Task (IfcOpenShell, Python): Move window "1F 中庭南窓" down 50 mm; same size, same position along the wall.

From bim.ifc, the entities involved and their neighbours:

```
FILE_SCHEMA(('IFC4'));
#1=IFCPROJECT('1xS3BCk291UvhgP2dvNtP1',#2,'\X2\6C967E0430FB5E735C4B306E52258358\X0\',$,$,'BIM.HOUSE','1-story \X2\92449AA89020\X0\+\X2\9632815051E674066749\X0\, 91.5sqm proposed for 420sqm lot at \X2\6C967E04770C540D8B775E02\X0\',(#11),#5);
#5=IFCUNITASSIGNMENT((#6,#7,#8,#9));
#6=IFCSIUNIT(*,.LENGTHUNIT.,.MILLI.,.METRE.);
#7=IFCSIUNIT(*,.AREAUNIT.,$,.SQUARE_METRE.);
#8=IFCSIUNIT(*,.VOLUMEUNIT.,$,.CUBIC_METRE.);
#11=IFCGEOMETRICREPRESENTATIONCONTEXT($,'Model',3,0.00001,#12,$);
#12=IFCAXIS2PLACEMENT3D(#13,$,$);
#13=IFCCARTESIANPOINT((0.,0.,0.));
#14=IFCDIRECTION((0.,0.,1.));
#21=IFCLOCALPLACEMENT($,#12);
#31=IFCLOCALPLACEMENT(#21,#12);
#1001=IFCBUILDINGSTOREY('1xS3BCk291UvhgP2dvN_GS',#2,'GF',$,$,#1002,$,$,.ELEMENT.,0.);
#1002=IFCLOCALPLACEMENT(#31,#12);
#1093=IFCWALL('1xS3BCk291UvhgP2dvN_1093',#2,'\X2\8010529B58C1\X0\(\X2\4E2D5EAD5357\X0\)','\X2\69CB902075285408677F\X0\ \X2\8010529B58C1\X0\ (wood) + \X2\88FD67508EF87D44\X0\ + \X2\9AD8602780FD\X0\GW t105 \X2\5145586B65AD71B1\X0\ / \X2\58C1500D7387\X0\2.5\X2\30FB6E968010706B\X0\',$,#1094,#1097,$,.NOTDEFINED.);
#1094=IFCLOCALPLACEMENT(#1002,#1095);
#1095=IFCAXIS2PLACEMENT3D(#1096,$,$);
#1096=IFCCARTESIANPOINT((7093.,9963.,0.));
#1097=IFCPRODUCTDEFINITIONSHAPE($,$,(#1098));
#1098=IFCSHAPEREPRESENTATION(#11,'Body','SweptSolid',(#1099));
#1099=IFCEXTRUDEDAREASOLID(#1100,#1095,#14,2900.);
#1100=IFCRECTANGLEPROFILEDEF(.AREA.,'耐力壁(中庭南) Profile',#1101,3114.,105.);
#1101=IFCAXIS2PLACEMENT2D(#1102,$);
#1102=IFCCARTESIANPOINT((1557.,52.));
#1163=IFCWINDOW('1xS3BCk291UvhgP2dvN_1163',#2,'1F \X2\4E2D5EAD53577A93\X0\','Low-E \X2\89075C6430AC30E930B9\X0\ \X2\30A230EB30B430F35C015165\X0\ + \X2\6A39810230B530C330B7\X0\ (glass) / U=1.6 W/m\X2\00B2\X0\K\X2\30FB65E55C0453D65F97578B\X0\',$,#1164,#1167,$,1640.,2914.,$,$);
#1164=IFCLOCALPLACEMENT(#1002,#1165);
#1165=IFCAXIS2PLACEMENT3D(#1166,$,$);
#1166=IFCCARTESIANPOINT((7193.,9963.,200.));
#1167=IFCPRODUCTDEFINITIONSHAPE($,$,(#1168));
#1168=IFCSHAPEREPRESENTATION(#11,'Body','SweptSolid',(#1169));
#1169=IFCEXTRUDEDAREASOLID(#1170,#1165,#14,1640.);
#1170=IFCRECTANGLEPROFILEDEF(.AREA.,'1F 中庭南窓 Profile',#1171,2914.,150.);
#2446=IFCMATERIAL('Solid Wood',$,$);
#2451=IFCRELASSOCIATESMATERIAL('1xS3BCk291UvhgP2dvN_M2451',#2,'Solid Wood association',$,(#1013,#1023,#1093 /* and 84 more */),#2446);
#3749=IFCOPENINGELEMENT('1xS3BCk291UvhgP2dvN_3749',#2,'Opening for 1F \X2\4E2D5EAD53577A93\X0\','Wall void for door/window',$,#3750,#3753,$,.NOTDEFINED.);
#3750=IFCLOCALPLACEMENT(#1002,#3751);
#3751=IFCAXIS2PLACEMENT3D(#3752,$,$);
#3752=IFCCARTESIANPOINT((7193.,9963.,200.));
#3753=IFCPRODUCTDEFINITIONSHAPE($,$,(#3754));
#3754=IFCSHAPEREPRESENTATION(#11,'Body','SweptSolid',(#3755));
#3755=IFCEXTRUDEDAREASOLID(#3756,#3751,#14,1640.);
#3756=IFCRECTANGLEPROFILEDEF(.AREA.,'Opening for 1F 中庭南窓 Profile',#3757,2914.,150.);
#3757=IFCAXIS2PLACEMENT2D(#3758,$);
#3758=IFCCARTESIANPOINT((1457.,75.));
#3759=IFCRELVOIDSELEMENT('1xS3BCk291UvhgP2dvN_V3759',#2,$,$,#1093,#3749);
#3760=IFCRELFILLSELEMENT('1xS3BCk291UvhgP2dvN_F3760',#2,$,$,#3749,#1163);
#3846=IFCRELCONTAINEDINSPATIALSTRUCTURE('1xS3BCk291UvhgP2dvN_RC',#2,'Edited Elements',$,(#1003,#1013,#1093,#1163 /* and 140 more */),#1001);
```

```python
import numpy as np
import ifcopenshell
import ifcopenshell.api.geometry
import ifcopenshell.util.placement
import ifcopenshell.util.unit

model = ifcopenshell.open("bim.ifc")
unit_scale = ifcopenshell.util.unit.calculate_unit_scale(model)

window = model.by_guid("1xS3BCk291UvhgP2dvN_1163")
opening = window.FillsVoids[0].RelatingOpeningElement
dz = -0.05 / unit_scale

shift = np.array([0.0, 0.0, dz])
# The window is not placed relative to its opening, so move both.
for product in (opening, window):
    matrix = ifcopenshell.util.placement.get_local_placement(product.ObjectPlacement)
    matrix[:3, 3] += shift
    ifcopenshell.api.geometry.edit_object_placement(model, product=product, matrix=matrix, is_si=False)

print(f"moved by {dz * unit_scale:+.3f} m")

model.write("bim_updated.ifc")
```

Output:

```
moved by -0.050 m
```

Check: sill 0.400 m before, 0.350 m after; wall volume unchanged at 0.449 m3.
